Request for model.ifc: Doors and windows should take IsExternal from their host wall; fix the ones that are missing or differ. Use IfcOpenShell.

First a look at what the model holds.

```python
import ifcopenshell
import ifcopenshell.util.element

model = ifcopenshell.open("model.ifc")
print(model.schema)
seen = {}
for e in model.by_type("IfcDoor") + model.by_type("IfcWindow"):
    if not e.FillsVoids:
        continue
    host = e.FillsVoids[0].RelatingOpeningElement.VoidsElements[0].RelatingBuildingElement
    own = ifcopenshell.util.element.get_pset(e, f"Pset_{e.is_a()[3:].removesuffix('StandardCase')}Common", "IsExternal")
    wall = ifcopenshell.util.element.get_pset(host, "Pset_WallCommon", "IsExternal")
    seen[e.is_a(), own, wall] = seen.get((e.is_a(), own, wall), 0) + 1
for (cls, own, wall), count in sorted(seen.items(), key=str):
    print(count, cls, "IsExternal:", own, "| host wall:", wall)
```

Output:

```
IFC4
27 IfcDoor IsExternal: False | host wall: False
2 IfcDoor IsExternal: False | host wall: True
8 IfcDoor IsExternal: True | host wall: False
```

```python
import ifcopenshell
import ifcopenshell.api.pset
import ifcopenshell.util.element

model = ifcopenshell.open("model.ifc")

count = 0
for ifc_class, pset_name in (("IfcDoor", "Pset_DoorCommon"), ("IfcWindow", "Pset_WindowCommon")):
    for e in model.by_type(ifc_class):
        if not e.FillsVoids:
            continue
        host = e.FillsVoids[0].RelatingOpeningElement.VoidsElements[0].RelatingBuildingElement
        external = ifcopenshell.util.element.get_pset(host, "Pset_WallCommon", "IsExternal")
        if external is None or ifcopenshell.util.element.get_pset(e, pset_name, "IsExternal") == external:
            continue
        pset = ifcopenshell.api.pset.add_pset(model, product=e, name=pset_name)
        ifcopenshell.api.pset.edit_pset(model, pset=pset, properties={"IsExternal": external})
        count += 1

print(count, "updated")

model.write("model_edited.ifc")
```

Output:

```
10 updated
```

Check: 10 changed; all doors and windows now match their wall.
